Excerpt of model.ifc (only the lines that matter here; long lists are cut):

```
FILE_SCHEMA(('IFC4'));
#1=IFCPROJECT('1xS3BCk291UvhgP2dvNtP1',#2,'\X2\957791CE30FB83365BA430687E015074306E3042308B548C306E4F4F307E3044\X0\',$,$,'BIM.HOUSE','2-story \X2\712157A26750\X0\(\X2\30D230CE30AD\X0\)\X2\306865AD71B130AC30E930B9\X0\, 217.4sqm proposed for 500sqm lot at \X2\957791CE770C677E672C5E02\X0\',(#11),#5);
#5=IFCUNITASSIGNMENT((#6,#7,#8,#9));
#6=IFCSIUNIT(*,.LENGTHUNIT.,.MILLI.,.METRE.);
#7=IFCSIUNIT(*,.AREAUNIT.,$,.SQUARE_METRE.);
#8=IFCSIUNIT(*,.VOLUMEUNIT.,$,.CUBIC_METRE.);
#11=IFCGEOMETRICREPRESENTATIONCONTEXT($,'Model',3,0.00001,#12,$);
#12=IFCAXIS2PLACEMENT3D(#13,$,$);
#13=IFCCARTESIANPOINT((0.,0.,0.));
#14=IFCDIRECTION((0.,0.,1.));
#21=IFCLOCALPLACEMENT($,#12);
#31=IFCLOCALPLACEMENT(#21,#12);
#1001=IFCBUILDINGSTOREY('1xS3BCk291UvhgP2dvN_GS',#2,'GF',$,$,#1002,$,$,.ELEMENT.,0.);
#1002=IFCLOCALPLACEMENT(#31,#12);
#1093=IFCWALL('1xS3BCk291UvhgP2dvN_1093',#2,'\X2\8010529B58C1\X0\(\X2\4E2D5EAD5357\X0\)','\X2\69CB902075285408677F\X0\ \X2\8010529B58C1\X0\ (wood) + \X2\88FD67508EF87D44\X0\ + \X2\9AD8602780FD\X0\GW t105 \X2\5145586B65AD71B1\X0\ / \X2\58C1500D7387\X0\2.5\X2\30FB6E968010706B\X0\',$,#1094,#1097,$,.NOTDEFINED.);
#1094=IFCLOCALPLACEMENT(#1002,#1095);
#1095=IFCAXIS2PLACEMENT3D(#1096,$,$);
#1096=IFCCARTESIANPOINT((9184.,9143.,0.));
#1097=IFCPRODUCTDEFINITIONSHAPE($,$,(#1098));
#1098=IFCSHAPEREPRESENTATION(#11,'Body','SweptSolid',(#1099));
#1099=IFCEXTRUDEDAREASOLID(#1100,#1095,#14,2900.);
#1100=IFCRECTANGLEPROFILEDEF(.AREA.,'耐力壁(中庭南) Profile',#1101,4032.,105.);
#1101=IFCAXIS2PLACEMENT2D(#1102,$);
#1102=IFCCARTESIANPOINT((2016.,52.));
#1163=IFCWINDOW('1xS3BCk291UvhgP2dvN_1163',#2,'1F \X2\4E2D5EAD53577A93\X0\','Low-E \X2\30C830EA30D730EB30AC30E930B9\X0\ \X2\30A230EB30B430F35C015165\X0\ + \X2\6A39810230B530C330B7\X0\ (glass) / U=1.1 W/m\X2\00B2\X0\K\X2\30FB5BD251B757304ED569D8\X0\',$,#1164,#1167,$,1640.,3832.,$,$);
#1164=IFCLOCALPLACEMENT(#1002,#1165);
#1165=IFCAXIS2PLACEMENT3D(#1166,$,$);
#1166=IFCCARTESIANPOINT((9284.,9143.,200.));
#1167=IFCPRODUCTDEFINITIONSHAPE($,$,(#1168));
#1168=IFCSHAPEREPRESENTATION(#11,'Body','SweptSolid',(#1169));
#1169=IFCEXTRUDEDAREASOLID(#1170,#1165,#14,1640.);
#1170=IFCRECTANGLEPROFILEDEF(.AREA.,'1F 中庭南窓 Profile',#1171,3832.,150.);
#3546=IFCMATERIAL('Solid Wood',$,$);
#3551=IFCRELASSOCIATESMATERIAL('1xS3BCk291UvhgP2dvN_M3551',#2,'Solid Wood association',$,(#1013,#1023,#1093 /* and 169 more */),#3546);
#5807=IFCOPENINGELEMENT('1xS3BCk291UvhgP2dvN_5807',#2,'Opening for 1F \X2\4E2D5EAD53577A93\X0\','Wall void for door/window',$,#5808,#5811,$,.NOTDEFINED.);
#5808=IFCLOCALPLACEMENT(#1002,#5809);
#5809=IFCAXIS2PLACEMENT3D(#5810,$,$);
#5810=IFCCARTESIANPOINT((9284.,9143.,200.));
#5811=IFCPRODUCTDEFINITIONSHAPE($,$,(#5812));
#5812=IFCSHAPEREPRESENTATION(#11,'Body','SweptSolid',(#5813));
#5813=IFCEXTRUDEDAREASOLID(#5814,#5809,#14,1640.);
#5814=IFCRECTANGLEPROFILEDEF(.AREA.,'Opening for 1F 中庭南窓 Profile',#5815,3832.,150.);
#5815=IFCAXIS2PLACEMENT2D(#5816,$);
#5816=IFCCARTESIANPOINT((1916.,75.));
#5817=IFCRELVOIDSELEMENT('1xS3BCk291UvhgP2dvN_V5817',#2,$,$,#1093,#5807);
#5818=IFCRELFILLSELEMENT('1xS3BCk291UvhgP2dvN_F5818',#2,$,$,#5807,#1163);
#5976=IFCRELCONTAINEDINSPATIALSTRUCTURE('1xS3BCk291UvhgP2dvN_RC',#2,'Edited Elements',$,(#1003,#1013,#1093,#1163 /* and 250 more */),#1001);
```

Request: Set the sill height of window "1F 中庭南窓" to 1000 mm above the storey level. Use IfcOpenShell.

```python
import numpy as np
import ifcopenshell
import ifcopenshell.api.geometry
import ifcopenshell.geom
import ifcopenshell.util.element
import ifcopenshell.util.placement
import ifcopenshell.util.shape
import ifcopenshell.util.unit

model = ifcopenshell.open("model.ifc")
unit_scale = ifcopenshell.util.unit.calculate_unit_scale(model)

window = model.by_guid("1xS3BCk291UvhgP2dvN_1163")
opening = window.FillsVoids[0].RelatingOpeningElement
storey = ifcopenshell.util.element.get_container(window, ifc_class="IfcBuildingStorey")
level = ifcopenshell.util.placement.get_local_placement(storey.ObjectPlacement)[2, 3]

# The opening's origin need not be at the sill, so measure its lowest point.
shape = ifcopenshell.geom.create_shape(ifcopenshell.geom.settings(), opening)
bottom = ifcopenshell.util.shape.get_shape_bottom_elevation(shape, shape.geometry) / unit_scale
dz = level + 1 / unit_scale - bottom

shift = np.array([0.0, 0.0, dz])
# The window is not placed relative to its opening, so move both.
for product in (opening, window):
    matrix = ifcopenshell.util.placement.get_local_placement(product.ObjectPlacement)
    matrix[:3, 3] += shift
    ifcopenshell.api.geometry.edit_object_placement(model, product=product, matrix=matrix, is_si=False)

print(f"moved by {dz * unit_scale:+.3f} m")

model.write("model_rev.ifc")
```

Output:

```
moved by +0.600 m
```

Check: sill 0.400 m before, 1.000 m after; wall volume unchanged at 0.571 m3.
